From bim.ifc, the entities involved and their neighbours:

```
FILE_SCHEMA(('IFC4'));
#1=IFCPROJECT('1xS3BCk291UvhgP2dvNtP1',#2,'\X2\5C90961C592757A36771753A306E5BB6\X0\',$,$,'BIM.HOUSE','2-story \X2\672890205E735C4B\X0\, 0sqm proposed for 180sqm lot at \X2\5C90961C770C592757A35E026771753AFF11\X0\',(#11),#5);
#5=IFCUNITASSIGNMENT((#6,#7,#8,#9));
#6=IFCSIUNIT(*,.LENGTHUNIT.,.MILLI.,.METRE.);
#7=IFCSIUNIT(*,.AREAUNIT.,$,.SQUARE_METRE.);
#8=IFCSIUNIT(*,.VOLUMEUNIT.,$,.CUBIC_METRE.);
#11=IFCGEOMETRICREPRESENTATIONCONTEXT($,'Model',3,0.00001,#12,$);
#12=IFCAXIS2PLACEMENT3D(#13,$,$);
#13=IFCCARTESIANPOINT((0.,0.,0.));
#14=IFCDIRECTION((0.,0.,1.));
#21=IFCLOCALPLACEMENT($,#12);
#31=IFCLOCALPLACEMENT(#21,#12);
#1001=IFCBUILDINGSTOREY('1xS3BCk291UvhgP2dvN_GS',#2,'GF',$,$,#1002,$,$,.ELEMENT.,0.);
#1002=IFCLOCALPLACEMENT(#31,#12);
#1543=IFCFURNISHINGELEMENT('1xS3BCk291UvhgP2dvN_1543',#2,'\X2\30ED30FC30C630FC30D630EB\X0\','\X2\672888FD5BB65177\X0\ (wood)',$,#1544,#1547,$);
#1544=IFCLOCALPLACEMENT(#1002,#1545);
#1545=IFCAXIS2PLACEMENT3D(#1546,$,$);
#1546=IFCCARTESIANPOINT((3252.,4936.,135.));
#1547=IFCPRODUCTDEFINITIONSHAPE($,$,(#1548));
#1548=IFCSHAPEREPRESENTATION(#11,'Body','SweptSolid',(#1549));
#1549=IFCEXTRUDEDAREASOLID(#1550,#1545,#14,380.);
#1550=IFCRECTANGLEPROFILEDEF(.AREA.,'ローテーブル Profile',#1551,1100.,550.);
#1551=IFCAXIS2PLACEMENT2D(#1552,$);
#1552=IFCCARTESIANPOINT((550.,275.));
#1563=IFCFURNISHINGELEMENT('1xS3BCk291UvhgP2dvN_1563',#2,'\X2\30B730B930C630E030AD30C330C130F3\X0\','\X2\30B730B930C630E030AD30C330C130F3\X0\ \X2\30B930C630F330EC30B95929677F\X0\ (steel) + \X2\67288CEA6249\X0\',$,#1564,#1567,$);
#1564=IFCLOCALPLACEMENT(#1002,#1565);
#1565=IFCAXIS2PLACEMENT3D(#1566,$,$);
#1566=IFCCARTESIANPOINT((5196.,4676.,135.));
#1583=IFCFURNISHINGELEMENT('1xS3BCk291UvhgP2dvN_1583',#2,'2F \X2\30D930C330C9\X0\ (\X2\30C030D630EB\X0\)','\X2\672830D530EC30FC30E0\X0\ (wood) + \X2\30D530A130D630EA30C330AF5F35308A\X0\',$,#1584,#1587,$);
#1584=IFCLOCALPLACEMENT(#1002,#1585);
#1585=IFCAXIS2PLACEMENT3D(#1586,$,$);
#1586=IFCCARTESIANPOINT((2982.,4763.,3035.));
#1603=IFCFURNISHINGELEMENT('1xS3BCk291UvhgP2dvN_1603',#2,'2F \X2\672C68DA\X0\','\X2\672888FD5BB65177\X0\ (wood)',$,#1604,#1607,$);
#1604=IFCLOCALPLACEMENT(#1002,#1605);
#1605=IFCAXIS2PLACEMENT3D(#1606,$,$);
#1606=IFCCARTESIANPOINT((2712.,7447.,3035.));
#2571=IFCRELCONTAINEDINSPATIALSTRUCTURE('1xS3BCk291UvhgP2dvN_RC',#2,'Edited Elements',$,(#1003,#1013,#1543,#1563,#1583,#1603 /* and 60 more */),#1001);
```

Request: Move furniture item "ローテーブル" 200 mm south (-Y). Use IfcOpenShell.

```python
import ifcopenshell
import ifcopenshell.api.geometry
import ifcopenshell.util.placement
import ifcopenshell.util.unit

model = ifcopenshell.open("bim.ifc")
unit_scale = ifcopenshell.util.unit.calculate_unit_scale(model)

item = model.by_guid("1xS3BCk291UvhgP2dvN_1543")
matrix = ifcopenshell.util.placement.get_local_placement(item.ObjectPlacement)
matrix[1, 3] -= 0.2 / unit_scale
ifcopenshell.api.geometry.edit_object_placement(model, product=item, matrix=matrix, is_si=False)

print(ifcopenshell.util.placement.get_local_placement(item.ObjectPlacement).round(3) + 0.0)

model.write("bim_updated.ifc")
```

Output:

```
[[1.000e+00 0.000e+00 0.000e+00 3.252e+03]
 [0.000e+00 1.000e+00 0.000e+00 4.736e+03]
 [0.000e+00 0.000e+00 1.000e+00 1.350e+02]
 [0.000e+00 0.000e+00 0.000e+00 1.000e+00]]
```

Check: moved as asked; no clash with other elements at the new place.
